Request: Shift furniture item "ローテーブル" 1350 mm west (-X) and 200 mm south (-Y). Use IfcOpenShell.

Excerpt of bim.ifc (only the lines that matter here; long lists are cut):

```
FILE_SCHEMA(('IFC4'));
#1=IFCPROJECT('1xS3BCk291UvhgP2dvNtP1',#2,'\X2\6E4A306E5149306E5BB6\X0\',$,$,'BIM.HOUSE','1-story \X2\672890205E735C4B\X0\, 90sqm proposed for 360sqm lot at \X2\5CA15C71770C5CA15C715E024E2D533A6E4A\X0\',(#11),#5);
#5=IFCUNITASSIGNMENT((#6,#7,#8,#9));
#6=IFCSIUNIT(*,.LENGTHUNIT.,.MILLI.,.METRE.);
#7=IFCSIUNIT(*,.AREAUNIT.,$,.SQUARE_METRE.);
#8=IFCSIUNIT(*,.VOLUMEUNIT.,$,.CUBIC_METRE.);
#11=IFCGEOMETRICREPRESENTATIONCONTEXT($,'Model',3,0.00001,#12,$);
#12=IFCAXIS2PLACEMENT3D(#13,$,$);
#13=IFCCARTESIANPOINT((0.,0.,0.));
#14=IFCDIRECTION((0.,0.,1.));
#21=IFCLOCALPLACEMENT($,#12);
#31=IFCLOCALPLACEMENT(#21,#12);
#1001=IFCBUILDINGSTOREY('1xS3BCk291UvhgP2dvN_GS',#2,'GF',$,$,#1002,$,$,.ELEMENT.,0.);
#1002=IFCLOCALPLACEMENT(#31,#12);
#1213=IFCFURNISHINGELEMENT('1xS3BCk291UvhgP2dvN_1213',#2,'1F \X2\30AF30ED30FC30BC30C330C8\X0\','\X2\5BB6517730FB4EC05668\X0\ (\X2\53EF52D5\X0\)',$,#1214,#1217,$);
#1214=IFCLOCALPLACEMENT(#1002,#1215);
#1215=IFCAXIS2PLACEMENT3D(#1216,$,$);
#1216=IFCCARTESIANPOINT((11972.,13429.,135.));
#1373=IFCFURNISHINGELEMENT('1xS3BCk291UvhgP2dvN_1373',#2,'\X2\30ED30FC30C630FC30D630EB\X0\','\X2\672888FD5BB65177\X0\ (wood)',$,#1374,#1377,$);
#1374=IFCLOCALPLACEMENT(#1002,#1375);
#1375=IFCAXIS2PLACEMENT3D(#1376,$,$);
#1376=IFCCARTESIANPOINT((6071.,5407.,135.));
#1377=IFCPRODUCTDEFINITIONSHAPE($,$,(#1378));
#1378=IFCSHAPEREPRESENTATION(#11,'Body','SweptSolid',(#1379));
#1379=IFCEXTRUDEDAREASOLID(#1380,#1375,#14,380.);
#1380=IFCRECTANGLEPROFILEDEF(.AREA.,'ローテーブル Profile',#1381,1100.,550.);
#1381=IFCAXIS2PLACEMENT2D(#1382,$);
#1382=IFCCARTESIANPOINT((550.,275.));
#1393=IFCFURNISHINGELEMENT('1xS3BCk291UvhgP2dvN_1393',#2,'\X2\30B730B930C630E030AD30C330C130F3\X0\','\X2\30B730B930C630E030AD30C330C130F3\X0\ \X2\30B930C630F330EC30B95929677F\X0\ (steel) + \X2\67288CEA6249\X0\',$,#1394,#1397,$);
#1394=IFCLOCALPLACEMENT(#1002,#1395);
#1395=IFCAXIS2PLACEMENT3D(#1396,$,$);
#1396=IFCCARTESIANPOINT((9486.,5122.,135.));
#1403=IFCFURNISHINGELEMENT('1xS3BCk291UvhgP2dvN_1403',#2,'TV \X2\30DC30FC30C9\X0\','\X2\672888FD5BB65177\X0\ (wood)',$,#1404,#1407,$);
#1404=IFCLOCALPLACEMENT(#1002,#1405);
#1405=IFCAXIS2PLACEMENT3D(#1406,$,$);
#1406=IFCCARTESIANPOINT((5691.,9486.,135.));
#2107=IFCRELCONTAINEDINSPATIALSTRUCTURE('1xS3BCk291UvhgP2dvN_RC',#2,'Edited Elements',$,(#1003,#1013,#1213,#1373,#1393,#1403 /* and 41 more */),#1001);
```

```python
import ifcopenshell
import ifcopenshell.api.geometry
import ifcopenshell.util.placement

model = ifcopenshell.open("bim.ifc")

item = model.by_guid("1xS3BCk291UvhgP2dvN_1373")
matrix = ifcopenshell.util.placement.get_local_placement(item.ObjectPlacement)
matrix[0, 3] -= 1350.0
matrix[1, 3] -= 200.0
ifcopenshell.api.geometry.edit_object_placement(model, product=item, matrix=matrix, is_si=False)

print(ifcopenshell.util.placement.get_local_placement(item.ObjectPlacement).round(3) + 0.0)

model.write("bim_v2.ifc")
```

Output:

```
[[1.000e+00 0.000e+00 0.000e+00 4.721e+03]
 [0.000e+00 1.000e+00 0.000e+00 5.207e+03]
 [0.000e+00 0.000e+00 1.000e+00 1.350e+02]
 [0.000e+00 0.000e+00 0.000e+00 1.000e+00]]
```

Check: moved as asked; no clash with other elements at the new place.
